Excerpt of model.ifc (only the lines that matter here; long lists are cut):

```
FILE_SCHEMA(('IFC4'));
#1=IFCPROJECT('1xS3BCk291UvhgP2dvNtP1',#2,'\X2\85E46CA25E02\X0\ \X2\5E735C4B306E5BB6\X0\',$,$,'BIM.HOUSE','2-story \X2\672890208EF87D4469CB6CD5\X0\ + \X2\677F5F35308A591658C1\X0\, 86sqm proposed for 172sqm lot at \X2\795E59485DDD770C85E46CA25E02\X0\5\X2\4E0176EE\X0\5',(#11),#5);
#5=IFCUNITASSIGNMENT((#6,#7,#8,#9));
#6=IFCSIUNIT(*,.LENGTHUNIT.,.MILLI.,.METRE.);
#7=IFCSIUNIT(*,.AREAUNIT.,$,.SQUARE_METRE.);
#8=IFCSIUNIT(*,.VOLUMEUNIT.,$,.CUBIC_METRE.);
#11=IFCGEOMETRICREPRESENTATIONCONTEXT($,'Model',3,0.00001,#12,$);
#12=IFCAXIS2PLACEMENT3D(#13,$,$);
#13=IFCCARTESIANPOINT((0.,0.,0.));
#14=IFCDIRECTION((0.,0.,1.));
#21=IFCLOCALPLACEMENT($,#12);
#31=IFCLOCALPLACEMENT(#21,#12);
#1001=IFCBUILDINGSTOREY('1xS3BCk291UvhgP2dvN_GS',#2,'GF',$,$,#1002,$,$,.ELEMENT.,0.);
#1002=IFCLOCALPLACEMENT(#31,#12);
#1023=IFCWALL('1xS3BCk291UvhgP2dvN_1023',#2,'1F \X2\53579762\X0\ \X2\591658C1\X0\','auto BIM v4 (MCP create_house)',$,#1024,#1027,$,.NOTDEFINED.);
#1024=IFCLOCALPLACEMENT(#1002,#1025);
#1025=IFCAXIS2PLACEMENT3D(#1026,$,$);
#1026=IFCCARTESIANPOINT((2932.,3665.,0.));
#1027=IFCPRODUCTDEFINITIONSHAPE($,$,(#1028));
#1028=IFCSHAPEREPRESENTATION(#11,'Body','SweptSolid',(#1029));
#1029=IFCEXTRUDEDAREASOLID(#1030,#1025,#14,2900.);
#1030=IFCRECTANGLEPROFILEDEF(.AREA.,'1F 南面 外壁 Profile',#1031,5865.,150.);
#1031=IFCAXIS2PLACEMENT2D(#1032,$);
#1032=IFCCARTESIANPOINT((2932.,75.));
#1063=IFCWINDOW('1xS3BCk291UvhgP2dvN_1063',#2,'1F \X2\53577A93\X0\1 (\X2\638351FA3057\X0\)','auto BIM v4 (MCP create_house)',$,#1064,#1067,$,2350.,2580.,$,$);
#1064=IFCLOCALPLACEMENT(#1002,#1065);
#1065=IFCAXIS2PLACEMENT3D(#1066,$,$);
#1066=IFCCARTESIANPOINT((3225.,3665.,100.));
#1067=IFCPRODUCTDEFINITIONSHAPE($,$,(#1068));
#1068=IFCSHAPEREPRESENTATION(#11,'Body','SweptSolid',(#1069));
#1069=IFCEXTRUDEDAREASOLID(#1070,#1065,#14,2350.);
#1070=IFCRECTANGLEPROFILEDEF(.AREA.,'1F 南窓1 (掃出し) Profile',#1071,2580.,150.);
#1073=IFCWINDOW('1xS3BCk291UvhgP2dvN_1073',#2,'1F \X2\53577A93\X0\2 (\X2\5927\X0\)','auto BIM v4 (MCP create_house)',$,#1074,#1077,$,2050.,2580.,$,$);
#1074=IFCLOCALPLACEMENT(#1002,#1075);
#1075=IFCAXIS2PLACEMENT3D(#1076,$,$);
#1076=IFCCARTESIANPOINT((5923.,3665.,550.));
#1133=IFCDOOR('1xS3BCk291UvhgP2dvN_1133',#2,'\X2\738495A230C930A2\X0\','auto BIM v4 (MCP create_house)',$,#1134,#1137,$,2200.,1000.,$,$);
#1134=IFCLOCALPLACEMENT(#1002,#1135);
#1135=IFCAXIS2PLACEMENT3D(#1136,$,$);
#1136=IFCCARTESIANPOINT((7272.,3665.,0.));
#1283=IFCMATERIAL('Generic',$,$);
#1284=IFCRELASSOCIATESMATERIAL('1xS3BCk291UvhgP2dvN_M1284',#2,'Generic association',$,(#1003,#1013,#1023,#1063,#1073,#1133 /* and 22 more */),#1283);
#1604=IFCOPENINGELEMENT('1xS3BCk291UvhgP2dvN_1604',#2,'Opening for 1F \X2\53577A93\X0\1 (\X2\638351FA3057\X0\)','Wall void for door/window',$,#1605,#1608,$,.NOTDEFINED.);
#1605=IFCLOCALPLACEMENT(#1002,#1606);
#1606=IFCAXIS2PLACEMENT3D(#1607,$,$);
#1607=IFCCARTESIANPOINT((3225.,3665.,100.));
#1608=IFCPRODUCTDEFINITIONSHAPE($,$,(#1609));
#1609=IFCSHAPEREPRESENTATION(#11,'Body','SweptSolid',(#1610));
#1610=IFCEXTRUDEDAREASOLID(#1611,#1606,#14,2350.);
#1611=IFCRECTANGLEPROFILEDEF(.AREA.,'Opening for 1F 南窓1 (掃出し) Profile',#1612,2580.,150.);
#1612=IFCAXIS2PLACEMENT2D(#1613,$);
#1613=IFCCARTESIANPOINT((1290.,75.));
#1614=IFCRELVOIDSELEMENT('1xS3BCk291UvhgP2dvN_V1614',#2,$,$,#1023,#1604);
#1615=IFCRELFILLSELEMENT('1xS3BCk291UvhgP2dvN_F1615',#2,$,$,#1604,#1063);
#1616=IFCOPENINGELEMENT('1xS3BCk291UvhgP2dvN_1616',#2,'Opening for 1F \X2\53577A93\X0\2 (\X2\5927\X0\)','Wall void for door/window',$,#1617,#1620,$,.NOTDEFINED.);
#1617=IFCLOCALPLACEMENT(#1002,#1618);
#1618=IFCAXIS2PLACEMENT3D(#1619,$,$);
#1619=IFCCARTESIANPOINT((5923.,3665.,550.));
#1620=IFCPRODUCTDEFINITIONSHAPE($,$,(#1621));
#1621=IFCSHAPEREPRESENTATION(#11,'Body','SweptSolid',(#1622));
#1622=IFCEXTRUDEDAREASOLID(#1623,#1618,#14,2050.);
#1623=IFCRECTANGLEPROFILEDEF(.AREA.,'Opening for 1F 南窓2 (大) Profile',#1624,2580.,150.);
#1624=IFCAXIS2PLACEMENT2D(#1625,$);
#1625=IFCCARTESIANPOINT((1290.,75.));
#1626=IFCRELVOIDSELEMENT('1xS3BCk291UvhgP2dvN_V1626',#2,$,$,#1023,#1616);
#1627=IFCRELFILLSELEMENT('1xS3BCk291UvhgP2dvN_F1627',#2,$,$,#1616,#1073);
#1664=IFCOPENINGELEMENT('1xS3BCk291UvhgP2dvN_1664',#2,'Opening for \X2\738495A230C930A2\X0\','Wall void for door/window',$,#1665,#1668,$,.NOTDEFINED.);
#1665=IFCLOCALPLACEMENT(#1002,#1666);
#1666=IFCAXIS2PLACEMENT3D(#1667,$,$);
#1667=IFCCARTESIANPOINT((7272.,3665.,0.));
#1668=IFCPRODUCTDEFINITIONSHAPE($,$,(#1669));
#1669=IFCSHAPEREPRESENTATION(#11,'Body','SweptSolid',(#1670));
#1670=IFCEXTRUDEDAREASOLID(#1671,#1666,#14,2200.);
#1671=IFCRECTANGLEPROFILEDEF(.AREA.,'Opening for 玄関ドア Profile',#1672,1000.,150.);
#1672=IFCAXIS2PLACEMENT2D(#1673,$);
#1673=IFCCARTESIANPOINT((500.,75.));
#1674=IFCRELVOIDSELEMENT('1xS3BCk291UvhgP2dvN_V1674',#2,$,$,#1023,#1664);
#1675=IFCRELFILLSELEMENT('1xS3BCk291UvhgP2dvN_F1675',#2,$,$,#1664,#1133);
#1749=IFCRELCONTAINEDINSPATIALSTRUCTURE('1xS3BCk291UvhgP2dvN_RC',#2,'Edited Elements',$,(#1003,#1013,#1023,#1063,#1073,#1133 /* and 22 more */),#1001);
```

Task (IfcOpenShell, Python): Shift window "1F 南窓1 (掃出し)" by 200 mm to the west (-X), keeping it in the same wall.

```python
import ifcopenshell
import ifcopenshell.api.geometry
import ifcopenshell.util.placement
import ifcopenshell.util.unit

model = ifcopenshell.open("model.ifc")
unit_scale = ifcopenshell.util.unit.calculate_unit_scale(model)

window = model.by_guid("1xS3BCk291UvhgP2dvN_1063")
opening = window.FillsVoids[0].RelatingOpeningElement
wall = opening.VoidsElements[0].RelatingBuildingElement

wall_matrix = ifcopenshell.util.placement.get_local_placement(wall.ObjectPlacement)
shift = wall_matrix[:3, 0] * -0.2 / unit_scale
before = ifcopenshell.util.placement.get_local_placement(window.ObjectPlacement)[:3, 3].copy()

# The window is not placed relative to its opening, so move both.
for product in (opening, window):
    matrix = ifcopenshell.util.placement.get_local_placement(product.ObjectPlacement)
    matrix[:3, 3] += shift
    ifcopenshell.api.geometry.edit_object_placement(model, product=product, matrix=matrix, is_si=False)

after = ifcopenshell.util.placement.get_local_placement(window.ObjectPlacement)[:3, 3]
print("window moved by", (after - before).round(3) + 0.0)

model.write("model_updated.ifc")
```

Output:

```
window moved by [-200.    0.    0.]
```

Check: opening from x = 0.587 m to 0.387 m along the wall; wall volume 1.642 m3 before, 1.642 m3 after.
